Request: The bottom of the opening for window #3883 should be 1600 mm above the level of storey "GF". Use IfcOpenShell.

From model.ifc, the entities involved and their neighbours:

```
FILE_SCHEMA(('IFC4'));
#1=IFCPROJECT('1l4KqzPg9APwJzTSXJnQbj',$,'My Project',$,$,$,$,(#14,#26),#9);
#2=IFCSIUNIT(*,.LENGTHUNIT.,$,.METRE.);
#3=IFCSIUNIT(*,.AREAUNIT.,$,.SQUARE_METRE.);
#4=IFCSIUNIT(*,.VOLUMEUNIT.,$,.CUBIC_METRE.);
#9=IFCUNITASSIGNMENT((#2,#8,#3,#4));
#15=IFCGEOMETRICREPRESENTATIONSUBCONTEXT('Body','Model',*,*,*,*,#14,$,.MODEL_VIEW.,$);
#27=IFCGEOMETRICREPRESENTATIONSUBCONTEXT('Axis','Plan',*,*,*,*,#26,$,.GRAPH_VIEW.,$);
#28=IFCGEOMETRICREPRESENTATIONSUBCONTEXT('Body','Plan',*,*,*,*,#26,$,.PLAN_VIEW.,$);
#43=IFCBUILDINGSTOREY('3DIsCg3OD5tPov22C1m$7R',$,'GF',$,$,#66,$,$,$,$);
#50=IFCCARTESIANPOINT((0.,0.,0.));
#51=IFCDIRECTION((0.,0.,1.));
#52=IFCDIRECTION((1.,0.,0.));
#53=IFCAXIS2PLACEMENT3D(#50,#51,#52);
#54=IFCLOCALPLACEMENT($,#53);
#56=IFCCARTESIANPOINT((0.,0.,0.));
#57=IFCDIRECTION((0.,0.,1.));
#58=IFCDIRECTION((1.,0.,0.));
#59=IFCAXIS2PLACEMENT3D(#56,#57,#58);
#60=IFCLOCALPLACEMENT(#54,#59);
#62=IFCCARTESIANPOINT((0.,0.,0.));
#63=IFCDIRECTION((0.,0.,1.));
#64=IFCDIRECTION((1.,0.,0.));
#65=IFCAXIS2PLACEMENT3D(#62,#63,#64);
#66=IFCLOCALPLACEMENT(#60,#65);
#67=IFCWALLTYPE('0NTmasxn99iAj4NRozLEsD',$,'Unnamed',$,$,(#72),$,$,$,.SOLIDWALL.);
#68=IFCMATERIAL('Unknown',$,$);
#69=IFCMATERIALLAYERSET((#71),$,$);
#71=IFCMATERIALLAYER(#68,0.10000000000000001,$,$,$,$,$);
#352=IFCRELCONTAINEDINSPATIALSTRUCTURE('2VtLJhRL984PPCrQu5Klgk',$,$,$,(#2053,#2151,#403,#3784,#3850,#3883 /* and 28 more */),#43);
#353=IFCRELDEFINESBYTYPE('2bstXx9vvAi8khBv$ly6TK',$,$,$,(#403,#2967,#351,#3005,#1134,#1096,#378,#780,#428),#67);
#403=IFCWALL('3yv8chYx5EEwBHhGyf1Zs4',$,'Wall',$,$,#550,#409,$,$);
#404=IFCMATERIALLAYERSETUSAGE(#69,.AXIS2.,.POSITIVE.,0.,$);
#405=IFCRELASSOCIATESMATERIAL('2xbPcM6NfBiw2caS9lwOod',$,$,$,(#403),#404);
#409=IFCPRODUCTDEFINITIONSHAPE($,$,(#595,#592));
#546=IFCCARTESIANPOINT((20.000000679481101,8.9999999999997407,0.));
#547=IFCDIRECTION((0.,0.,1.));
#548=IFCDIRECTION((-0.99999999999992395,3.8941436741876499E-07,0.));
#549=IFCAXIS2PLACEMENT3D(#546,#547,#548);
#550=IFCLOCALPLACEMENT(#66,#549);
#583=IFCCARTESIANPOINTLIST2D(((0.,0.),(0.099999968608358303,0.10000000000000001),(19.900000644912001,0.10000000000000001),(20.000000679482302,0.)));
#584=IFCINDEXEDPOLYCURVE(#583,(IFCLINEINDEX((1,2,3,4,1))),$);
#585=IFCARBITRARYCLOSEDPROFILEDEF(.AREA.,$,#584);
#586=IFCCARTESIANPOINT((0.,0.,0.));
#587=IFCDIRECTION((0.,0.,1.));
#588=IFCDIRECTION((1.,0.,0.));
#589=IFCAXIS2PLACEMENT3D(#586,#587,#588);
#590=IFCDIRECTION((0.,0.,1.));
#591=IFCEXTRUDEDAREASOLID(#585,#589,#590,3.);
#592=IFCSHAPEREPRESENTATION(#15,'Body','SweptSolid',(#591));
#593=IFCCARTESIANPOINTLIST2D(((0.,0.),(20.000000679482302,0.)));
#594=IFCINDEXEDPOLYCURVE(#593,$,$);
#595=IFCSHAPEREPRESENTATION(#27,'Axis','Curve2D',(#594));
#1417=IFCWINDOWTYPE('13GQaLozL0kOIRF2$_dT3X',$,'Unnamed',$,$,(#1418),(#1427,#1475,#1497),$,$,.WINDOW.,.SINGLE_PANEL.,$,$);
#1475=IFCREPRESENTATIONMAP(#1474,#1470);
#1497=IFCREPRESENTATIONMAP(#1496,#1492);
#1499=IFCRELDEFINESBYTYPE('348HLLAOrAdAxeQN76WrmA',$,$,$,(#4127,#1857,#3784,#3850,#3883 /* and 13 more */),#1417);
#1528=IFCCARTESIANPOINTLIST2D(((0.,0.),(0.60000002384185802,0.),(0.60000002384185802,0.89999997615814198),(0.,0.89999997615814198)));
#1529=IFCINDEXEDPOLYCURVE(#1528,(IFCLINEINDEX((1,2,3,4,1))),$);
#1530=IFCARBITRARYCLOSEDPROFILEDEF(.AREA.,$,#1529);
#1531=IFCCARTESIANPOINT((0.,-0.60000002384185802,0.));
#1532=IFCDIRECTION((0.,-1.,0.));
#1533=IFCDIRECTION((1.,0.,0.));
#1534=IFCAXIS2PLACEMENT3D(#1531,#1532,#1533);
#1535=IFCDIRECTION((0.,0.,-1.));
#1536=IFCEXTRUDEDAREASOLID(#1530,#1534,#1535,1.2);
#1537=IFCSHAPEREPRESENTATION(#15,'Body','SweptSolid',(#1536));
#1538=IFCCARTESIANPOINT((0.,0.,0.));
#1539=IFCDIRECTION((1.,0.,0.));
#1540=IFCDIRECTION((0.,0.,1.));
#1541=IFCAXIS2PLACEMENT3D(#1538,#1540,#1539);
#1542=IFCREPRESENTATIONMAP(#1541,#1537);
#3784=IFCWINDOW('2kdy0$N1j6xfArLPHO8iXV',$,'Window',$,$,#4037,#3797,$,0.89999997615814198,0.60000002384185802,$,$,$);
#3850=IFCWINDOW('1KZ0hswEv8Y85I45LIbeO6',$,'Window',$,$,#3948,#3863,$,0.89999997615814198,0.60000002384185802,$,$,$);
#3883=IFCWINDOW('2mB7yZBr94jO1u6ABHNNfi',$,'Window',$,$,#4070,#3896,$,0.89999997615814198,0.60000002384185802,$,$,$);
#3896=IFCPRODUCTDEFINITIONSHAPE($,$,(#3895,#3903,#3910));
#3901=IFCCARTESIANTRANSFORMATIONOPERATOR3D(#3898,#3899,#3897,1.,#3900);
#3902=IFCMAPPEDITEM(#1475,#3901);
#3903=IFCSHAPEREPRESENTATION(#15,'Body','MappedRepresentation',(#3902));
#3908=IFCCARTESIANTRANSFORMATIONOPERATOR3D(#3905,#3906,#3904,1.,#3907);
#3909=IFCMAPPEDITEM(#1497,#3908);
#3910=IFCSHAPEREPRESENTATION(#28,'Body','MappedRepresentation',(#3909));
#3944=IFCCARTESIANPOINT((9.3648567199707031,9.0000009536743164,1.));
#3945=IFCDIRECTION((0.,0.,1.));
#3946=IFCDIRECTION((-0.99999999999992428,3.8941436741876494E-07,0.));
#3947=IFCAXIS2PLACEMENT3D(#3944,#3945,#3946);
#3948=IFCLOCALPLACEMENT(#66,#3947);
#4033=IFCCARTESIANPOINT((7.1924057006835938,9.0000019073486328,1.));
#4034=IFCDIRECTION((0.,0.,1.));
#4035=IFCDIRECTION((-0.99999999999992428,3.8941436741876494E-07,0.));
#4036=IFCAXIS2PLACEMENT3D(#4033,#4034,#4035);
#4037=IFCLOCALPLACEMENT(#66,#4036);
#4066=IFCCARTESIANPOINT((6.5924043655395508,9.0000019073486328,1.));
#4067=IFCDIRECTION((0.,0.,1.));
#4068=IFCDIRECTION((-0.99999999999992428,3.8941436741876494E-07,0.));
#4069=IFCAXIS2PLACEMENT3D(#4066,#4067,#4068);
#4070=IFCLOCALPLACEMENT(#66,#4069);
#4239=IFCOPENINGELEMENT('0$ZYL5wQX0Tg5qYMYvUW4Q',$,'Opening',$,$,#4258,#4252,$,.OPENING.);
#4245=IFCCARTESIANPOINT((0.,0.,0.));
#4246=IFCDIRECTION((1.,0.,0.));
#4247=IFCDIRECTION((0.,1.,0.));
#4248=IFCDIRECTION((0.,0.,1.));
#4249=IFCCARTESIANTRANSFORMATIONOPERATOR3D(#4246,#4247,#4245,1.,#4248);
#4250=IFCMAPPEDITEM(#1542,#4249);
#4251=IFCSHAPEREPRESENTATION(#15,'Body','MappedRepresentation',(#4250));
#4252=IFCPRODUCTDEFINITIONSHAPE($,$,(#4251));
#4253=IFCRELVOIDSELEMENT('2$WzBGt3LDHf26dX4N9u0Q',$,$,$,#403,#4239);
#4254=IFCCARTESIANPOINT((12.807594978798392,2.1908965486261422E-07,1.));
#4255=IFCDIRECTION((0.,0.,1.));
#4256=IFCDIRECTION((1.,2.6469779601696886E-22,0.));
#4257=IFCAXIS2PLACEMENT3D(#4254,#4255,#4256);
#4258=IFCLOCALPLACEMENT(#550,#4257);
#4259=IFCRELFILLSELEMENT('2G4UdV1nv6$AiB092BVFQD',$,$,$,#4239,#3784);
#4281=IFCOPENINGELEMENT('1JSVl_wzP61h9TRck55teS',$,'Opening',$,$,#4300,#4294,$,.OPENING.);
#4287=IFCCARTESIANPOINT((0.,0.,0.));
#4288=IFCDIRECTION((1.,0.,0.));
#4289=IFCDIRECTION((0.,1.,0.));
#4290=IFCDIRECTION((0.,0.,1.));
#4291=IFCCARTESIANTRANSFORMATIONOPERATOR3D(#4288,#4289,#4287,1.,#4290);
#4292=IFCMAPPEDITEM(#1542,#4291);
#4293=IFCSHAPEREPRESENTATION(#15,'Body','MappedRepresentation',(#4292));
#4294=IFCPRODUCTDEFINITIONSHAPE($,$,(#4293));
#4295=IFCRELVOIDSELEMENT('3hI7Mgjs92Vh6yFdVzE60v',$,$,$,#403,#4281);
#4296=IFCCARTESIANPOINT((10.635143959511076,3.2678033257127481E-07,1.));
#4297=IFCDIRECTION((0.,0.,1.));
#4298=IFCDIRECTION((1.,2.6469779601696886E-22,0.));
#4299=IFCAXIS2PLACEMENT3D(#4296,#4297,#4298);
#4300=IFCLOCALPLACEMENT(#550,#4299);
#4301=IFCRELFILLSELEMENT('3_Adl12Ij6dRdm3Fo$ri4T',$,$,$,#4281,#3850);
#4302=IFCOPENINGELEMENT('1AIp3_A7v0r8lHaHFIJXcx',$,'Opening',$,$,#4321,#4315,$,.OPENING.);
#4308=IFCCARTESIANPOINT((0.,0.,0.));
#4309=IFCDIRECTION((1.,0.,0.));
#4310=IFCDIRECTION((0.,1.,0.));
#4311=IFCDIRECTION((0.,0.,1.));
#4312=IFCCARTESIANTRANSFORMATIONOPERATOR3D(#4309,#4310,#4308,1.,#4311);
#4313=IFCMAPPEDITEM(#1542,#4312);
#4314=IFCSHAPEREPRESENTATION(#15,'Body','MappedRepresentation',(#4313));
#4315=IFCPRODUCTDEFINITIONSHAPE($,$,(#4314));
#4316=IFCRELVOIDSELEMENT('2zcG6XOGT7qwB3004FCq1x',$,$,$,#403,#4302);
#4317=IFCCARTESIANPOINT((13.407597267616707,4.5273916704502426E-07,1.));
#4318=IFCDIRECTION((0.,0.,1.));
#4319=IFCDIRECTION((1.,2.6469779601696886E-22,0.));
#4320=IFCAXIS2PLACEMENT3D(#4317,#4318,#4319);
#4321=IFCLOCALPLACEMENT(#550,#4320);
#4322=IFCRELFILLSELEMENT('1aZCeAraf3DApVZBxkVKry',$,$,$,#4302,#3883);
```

```python
import numpy as np
import ifcopenshell
import ifcopenshell.api.geometry
import ifcopenshell.geom
import ifcopenshell.util.element
import ifcopenshell.util.placement
import ifcopenshell.util.shape
import ifcopenshell.util.unit

model = ifcopenshell.open("model.ifc")
unit_scale = ifcopenshell.util.unit.calculate_unit_scale(model)

window = model.by_id(3883)
opening = window.FillsVoids[0].RelatingOpeningElement
storey = ifcopenshell.util.element.get_container(window, ifc_class="IfcBuildingStorey")
level = ifcopenshell.util.placement.get_local_placement(storey.ObjectPlacement)[2, 3]

# The opening's origin need not be at the sill, so measure its lowest point.
shape = ifcopenshell.geom.create_shape(ifcopenshell.geom.settings(), opening)
bottom = ifcopenshell.util.shape.get_shape_bottom_elevation(shape, shape.geometry) / unit_scale
dz = level + 1.6 - bottom

shift = np.array([0.0, 0.0, dz])
# The window is not placed relative to its opening, so move both.
for product in (opening, window):
    matrix = ifcopenshell.util.placement.get_local_placement(product.ObjectPlacement)
    matrix[:3, 3] += shift
    ifcopenshell.api.geometry.edit_object_placement(model, product=product, matrix=matrix, is_si=False)

print(f"moved by {dz * unit_scale:+.3f} m")

model.write("model-out.ifc")
```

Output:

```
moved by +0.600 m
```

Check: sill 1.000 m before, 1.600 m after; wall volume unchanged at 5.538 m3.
